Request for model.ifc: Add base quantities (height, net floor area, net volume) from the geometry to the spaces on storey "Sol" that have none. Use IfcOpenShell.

First a look at what the model holds.

```python
import ifcopenshell
import ifcopenshell.util.element
import ifcopenshell.util.unit

model = ifcopenshell.open("model.ifc")
print(model.schema)
for unit_type in ("LENGTHUNIT", "AREAUNIT", "VOLUMEUNIT"):
    print(unit_type, ifcopenshell.util.unit.calculate_unit_scale(model, unit_type))
storey = next(s for s in model.by_type("IfcBuildingStorey") if s.Name == "Sol")
spaces = [e for e in ifcopenshell.util.element.get_decomposition(storey) if e.is_a("IfcSpace")]
for e in sorted(spaces, key=lambda e: e.id()):
    print(e.id(), e.is_a(), e.Name, list(ifcopenshell.util.element.get_psets(e, qtos_only=True)), sep=" | ")
```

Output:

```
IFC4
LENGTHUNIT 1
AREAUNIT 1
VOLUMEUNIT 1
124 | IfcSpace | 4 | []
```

```python
import ifcopenshell
import ifcopenshell.api.pset
import ifcopenshell.geom
import ifcopenshell.util.element
import ifcopenshell.util.shape
import ifcopenshell.util.unit

model = ifcopenshell.open("model.ifc")
unit_scale = ifcopenshell.util.unit.calculate_unit_scale(model)
area_scale = ifcopenshell.util.unit.calculate_unit_scale(model, "AREAUNIT")
volume_scale = ifcopenshell.util.unit.calculate_unit_scale(model, "VOLUMEUNIT")
settings = ifcopenshell.geom.settings()

storey = next(s for s in model.by_type("IfcBuildingStorey") if s.Name == "Sol")
spaces = [e for e in ifcopenshell.util.element.get_decomposition(storey) if e.is_a("IfcSpace")]

for e in sorted(spaces, key=lambda e: e.id()):
    if ifcopenshell.util.element.get_psets(e, qtos_only=True, should_inherit=False):
        continue
    # Geometry comes back in metres, in the element's own axes.
    shape = ifcopenshell.geom.create_shape(settings, e)
    values = {
        "Height": ifcopenshell.util.shape.get_z(shape.geometry) / unit_scale,
        "NetFloorArea": ifcopenshell.util.shape.get_footprint_area(shape.geometry) / area_scale,
        "NetVolume": ifcopenshell.util.shape.get_volume(shape.geometry) / volume_scale,
    }
    qto = ifcopenshell.api.pset.add_qto(model, product=e, name="Qto_SpaceBaseQuantities")
    ifcopenshell.api.pset.edit_qto(model, qto=qto, properties=values)
    print(e.id(), {k: round(v, 3) for k, v in values.items()})

model.write("model_edited.ifc")
```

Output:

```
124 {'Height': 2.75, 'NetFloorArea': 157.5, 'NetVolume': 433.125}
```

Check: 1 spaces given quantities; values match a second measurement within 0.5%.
